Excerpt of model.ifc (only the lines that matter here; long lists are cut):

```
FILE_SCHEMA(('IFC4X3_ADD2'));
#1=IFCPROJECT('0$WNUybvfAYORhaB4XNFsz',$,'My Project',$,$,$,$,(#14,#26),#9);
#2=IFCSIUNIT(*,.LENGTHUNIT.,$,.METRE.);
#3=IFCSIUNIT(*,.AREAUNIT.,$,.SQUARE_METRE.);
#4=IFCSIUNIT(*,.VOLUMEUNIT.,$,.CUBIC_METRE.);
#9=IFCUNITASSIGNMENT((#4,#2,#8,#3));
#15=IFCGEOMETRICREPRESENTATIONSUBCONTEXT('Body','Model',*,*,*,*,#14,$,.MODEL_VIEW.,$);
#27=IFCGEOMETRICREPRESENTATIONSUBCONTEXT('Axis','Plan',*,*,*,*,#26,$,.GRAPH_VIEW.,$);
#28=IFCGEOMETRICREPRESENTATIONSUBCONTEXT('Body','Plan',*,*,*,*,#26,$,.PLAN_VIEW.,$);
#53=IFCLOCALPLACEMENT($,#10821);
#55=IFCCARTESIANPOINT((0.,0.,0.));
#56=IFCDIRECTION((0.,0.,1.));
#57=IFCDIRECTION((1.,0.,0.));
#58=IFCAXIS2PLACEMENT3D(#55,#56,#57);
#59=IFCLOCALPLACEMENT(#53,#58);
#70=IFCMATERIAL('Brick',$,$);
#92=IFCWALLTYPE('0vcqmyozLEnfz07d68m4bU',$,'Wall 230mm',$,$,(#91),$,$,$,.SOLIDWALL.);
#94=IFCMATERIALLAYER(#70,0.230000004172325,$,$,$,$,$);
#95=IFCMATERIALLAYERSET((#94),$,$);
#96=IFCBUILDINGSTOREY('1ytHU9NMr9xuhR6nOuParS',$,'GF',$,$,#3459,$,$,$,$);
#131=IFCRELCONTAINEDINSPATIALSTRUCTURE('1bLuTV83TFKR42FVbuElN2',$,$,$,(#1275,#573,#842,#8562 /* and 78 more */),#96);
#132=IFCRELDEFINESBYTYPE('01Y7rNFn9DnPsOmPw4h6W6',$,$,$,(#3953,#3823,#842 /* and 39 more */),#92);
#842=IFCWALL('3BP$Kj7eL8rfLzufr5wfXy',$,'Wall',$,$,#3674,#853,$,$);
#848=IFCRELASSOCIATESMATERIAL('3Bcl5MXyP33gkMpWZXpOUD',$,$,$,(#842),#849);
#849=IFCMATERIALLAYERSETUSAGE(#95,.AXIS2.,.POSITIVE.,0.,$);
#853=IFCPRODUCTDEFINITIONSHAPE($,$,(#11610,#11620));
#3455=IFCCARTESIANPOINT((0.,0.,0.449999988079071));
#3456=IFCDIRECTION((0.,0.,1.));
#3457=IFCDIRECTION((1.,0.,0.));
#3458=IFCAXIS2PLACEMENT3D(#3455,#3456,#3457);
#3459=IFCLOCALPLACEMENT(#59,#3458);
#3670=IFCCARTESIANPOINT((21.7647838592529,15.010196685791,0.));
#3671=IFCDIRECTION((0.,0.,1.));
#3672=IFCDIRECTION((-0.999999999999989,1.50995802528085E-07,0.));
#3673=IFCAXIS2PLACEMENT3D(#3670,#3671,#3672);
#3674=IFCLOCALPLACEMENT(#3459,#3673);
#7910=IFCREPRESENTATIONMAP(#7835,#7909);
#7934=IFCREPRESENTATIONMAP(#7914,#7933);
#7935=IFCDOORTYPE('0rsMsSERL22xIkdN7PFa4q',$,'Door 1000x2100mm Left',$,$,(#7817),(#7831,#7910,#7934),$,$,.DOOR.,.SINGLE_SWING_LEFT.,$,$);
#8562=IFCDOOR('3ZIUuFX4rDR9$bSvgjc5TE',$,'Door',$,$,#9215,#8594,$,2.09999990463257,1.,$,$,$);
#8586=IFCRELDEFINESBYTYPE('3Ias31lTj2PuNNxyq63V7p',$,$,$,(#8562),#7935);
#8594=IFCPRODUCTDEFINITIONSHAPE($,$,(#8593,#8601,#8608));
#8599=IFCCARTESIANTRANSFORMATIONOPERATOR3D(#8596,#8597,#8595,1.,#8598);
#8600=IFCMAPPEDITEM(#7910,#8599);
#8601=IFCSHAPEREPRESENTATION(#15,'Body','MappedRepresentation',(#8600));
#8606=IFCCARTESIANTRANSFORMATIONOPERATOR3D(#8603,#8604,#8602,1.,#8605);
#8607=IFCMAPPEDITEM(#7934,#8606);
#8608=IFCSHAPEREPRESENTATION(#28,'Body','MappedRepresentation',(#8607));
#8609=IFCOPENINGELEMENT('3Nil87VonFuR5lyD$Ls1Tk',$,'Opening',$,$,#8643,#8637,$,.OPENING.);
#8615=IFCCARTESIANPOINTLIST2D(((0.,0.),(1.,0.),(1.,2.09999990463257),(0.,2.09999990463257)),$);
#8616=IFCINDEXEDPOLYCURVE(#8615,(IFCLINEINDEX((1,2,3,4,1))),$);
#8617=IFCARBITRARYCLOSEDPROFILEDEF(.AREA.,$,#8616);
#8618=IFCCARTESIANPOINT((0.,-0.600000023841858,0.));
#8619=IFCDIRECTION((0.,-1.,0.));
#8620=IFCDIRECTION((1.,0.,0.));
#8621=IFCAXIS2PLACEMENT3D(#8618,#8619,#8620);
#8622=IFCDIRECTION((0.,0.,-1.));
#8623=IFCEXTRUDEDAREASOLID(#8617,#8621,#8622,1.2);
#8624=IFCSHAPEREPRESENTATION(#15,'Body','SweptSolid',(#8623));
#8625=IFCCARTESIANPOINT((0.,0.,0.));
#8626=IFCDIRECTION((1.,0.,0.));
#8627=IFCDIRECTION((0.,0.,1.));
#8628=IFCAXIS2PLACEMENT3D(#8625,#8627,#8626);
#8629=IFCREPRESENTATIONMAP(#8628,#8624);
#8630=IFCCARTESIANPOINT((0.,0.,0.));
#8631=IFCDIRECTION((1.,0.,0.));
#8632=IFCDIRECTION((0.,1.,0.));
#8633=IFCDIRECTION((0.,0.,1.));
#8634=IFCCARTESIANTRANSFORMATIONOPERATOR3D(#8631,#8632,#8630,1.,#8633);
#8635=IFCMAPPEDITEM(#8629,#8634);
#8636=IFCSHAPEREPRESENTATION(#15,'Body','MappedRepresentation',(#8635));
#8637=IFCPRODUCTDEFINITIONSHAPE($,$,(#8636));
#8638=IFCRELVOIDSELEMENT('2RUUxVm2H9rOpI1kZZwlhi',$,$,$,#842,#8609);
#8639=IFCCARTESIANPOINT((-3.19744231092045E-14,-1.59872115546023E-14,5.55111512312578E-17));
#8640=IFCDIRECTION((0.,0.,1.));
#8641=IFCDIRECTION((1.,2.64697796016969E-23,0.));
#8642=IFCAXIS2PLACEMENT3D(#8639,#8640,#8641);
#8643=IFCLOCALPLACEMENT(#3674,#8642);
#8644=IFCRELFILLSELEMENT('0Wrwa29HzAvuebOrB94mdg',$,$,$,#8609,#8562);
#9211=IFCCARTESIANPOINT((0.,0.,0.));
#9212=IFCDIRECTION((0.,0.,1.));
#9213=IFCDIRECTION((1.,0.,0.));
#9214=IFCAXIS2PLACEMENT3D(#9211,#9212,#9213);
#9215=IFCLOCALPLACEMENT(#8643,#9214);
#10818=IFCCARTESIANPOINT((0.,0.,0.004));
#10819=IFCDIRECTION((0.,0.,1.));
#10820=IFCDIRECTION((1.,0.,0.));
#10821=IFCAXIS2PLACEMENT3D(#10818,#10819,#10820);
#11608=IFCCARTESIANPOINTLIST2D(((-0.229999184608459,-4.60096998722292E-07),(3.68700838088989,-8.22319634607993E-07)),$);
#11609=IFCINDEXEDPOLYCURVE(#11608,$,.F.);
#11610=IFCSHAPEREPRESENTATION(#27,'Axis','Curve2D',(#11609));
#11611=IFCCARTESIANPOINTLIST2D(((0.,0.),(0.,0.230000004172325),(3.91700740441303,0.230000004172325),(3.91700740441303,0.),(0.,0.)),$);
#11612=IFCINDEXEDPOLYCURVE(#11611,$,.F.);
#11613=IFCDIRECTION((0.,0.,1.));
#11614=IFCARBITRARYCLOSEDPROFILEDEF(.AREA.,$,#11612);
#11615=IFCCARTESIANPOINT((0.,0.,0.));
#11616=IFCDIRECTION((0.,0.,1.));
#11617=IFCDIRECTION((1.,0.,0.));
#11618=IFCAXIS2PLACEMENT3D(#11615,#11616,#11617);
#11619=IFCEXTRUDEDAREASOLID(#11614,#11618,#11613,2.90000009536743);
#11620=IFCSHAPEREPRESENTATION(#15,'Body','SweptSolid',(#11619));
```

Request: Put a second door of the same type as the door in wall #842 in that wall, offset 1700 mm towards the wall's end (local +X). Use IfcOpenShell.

```python
import ifcopenshell
import ifcopenshell.api.feature
import ifcopenshell.api.geometry
import ifcopenshell.api.root
import ifcopenshell.geom
import ifcopenshell.util.element
import ifcopenshell.util.placement
import ifcopenshell.util.shape
import ifcopenshell.util.unit

model = ifcopenshell.open("model.ifc")
unit_scale = ifcopenshell.util.unit.calculate_unit_scale(model)
settings = ifcopenshell.geom.settings()


def volume(element):
    """Net volume in cubic metres, openings subtracted."""
    shape = ifcopenshell.geom.create_shape(settings, element)
    return ifcopenshell.util.shape.get_volume(shape.geometry)


door = model.by_guid("3ZIUuFX4rDR9$bSvgjc5TE")
opening = door.FillsVoids[0].RelatingOpeningElement
wall = opening.VoidsElements[0].RelatingBuildingElement
before = volume(wall)
shift = ifcopenshell.util.placement.get_local_placement(wall.ObjectPlacement)[:3, 0] * 1.7 / unit_scale

# copy_class copies the void relationship, type, container and properties, but no geometry.
new_opening = ifcopenshell.api.root.copy_class(model, product=opening)
new_opening.Representation = ifcopenshell.util.element.copy_deep(
    model, opening.Representation, exclude=["IfcGeometricRepresentationContext", "IfcRepresentationMap"]
)
new_door = ifcopenshell.api.root.copy_class(model, product=door)
new_door.Representation = ifcopenshell.util.element.copy_deep(
    model, door.Representation, exclude=["IfcGeometricRepresentationContext", "IfcRepresentationMap"]
)
ifcopenshell.api.feature.add_filling(model, opening=new_opening, element=new_door)

for old, new in ((opening, new_opening), (door, new_door)):
    matrix = ifcopenshell.util.placement.get_local_placement(old.ObjectPlacement)
    matrix[:3, 3] += shift
    ifcopenshell.api.geometry.edit_object_placement(model, product=new, matrix=matrix, is_si=False)

after = volume(wall)

print(f"wall volume {before:.3f} -> {after:.3f} m3")

model.write("model_edited.ifc")
```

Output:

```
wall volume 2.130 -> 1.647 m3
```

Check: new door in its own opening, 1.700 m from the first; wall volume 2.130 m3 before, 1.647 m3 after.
